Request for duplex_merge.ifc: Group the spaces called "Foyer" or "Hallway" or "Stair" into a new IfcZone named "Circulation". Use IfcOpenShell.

First a look at what the model holds.

```python
import ifcopenshell

model = ifcopenshell.open("duplex_merge.ifc")
print(model.schema)
seen = {}
for space in model.by_type("IfcSpace"):
    seen[space.LongName] = seen.get(space.LongName, 0) + 1
for name, count in sorted(seen.items(), key=str):
    print(count, "x", name)
print("zones:", [z.Name for z in model.by_type("IfcZone")][:20])
```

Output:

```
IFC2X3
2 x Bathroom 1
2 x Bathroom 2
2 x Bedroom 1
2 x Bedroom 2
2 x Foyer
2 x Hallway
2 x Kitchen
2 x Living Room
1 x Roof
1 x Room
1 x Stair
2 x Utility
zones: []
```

```python
import ifcopenshell
import ifcopenshell.api.group
import ifcopenshell.api.root

model = ifcopenshell.open("duplex_merge.ifc")

names = {"Foyer", "Hallway", "Stair"}
spaces = [s for s in model.by_type("IfcSpace") if s.LongName in names]

zone = ifcopenshell.api.root.create_entity(model, ifc_class="IfcZone", name="Circulation")
ifcopenshell.api.group.assign_group(model, products=spaces, group=zone)
print(len(spaces), "spaces in", zone.Name)

model.write("duplex_merge_v2.ifc")
```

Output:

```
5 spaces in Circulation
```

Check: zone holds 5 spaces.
